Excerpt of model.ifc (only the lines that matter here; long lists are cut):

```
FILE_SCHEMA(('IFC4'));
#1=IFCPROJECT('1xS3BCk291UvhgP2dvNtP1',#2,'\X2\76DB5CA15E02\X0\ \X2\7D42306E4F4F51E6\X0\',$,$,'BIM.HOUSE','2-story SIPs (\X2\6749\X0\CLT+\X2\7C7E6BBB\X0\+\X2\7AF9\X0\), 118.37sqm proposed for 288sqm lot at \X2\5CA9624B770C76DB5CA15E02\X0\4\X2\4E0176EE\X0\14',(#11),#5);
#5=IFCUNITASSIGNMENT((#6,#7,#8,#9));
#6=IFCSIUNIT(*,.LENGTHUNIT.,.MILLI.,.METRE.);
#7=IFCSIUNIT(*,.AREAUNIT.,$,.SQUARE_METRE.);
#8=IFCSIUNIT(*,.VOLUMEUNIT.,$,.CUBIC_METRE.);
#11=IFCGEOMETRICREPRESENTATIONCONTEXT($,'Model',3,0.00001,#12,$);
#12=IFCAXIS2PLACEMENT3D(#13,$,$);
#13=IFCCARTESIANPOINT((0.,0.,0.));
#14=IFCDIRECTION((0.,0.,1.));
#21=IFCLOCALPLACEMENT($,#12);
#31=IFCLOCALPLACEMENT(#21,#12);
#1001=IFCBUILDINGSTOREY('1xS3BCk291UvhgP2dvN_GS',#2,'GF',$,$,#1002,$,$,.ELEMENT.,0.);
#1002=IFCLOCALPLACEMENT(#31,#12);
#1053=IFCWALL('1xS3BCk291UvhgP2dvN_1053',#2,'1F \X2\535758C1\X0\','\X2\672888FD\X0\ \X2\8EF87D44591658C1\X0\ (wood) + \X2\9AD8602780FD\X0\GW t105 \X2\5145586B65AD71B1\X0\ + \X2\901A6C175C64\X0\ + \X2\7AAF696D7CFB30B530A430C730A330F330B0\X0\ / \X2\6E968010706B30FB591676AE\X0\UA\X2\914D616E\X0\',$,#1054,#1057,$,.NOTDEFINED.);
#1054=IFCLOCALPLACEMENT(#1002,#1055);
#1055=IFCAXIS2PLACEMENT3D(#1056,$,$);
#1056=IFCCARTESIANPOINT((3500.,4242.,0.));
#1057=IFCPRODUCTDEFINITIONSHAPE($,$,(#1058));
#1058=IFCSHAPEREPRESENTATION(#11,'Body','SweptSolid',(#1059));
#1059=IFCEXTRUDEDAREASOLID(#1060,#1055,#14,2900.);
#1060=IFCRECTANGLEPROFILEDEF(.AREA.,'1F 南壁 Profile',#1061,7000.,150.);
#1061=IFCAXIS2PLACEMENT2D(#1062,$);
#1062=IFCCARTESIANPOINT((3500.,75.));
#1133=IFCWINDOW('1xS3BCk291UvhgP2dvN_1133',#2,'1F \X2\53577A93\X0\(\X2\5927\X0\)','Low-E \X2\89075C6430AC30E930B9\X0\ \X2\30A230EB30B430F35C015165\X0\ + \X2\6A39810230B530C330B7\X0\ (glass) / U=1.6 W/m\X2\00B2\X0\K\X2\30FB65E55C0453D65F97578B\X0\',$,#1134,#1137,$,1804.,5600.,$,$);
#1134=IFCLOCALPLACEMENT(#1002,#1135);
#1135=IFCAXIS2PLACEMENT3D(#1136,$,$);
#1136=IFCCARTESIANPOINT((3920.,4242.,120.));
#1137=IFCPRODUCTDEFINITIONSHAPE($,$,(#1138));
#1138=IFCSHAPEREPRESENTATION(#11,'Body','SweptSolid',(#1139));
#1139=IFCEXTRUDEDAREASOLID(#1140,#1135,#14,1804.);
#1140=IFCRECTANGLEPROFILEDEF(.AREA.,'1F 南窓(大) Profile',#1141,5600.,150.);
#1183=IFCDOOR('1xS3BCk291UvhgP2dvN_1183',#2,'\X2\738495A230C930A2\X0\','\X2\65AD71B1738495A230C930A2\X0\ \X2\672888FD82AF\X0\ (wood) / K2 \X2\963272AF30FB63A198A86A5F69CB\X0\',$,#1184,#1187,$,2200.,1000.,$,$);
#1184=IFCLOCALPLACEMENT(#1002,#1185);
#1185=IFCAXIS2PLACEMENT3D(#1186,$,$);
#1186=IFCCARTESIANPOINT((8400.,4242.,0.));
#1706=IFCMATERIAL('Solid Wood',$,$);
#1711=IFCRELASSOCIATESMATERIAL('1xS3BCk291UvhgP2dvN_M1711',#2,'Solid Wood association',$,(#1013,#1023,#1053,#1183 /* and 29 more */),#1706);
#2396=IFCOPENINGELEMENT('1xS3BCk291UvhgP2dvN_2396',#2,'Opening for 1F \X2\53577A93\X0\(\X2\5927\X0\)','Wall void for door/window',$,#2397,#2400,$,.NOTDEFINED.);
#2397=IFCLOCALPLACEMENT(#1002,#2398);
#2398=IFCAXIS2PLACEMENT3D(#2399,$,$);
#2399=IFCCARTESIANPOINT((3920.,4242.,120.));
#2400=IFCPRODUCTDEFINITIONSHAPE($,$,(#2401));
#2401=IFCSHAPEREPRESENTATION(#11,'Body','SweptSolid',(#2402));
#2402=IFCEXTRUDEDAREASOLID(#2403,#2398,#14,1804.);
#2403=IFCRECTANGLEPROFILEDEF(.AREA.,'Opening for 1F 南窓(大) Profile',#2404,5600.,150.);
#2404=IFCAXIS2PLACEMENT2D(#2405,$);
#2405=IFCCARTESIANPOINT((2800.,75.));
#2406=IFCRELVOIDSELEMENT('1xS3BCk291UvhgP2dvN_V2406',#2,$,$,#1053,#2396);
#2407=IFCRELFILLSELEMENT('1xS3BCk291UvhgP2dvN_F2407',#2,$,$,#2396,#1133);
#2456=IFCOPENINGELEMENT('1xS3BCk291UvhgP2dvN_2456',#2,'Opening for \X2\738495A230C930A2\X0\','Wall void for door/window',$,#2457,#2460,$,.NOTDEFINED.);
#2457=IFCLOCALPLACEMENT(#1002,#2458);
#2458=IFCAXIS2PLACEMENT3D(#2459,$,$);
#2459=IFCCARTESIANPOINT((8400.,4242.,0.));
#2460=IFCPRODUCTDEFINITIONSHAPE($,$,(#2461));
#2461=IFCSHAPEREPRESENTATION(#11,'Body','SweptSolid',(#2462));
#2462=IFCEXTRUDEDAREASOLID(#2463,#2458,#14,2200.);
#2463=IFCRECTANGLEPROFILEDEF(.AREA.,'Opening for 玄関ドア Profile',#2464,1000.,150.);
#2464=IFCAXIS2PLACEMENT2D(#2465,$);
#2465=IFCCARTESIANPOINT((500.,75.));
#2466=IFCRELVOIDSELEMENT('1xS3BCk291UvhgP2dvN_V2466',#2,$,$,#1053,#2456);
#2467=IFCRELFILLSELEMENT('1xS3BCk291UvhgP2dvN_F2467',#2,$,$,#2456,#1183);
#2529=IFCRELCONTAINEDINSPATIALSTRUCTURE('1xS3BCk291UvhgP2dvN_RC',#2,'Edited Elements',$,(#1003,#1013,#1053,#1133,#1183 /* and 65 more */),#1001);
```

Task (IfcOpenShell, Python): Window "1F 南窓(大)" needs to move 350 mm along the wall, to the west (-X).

```python
import ifcopenshell
import ifcopenshell.api.geometry
import ifcopenshell.util.placement
import ifcopenshell.util.unit

model = ifcopenshell.open("model.ifc")
unit_scale = ifcopenshell.util.unit.calculate_unit_scale(model)

window = model.by_guid("1xS3BCk291UvhgP2dvN_1133")
opening = window.FillsVoids[0].RelatingOpeningElement
wall = opening.VoidsElements[0].RelatingBuildingElement

wall_matrix = ifcopenshell.util.placement.get_local_placement(wall.ObjectPlacement)
shift = wall_matrix[:3, 0] * -0.35 / unit_scale
before = ifcopenshell.util.placement.get_local_placement(window.ObjectPlacement)[:3, 3].copy()

# The window is not placed relative to its opening, so move both.
for product in (opening, window):
    matrix = ifcopenshell.util.placement.get_local_placement(product.ObjectPlacement)
    matrix[:3, 3] += shift
    ifcopenshell.api.geometry.edit_object_placement(model, product=product, matrix=matrix, is_si=False)

after = ifcopenshell.util.placement.get_local_placement(window.ObjectPlacement)[:3, 3]
print("window moved by", (after - before).round(3) + 0.0)

model.write("model_v2.ifc")
```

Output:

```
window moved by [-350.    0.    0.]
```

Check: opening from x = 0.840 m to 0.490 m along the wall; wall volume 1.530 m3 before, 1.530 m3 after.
